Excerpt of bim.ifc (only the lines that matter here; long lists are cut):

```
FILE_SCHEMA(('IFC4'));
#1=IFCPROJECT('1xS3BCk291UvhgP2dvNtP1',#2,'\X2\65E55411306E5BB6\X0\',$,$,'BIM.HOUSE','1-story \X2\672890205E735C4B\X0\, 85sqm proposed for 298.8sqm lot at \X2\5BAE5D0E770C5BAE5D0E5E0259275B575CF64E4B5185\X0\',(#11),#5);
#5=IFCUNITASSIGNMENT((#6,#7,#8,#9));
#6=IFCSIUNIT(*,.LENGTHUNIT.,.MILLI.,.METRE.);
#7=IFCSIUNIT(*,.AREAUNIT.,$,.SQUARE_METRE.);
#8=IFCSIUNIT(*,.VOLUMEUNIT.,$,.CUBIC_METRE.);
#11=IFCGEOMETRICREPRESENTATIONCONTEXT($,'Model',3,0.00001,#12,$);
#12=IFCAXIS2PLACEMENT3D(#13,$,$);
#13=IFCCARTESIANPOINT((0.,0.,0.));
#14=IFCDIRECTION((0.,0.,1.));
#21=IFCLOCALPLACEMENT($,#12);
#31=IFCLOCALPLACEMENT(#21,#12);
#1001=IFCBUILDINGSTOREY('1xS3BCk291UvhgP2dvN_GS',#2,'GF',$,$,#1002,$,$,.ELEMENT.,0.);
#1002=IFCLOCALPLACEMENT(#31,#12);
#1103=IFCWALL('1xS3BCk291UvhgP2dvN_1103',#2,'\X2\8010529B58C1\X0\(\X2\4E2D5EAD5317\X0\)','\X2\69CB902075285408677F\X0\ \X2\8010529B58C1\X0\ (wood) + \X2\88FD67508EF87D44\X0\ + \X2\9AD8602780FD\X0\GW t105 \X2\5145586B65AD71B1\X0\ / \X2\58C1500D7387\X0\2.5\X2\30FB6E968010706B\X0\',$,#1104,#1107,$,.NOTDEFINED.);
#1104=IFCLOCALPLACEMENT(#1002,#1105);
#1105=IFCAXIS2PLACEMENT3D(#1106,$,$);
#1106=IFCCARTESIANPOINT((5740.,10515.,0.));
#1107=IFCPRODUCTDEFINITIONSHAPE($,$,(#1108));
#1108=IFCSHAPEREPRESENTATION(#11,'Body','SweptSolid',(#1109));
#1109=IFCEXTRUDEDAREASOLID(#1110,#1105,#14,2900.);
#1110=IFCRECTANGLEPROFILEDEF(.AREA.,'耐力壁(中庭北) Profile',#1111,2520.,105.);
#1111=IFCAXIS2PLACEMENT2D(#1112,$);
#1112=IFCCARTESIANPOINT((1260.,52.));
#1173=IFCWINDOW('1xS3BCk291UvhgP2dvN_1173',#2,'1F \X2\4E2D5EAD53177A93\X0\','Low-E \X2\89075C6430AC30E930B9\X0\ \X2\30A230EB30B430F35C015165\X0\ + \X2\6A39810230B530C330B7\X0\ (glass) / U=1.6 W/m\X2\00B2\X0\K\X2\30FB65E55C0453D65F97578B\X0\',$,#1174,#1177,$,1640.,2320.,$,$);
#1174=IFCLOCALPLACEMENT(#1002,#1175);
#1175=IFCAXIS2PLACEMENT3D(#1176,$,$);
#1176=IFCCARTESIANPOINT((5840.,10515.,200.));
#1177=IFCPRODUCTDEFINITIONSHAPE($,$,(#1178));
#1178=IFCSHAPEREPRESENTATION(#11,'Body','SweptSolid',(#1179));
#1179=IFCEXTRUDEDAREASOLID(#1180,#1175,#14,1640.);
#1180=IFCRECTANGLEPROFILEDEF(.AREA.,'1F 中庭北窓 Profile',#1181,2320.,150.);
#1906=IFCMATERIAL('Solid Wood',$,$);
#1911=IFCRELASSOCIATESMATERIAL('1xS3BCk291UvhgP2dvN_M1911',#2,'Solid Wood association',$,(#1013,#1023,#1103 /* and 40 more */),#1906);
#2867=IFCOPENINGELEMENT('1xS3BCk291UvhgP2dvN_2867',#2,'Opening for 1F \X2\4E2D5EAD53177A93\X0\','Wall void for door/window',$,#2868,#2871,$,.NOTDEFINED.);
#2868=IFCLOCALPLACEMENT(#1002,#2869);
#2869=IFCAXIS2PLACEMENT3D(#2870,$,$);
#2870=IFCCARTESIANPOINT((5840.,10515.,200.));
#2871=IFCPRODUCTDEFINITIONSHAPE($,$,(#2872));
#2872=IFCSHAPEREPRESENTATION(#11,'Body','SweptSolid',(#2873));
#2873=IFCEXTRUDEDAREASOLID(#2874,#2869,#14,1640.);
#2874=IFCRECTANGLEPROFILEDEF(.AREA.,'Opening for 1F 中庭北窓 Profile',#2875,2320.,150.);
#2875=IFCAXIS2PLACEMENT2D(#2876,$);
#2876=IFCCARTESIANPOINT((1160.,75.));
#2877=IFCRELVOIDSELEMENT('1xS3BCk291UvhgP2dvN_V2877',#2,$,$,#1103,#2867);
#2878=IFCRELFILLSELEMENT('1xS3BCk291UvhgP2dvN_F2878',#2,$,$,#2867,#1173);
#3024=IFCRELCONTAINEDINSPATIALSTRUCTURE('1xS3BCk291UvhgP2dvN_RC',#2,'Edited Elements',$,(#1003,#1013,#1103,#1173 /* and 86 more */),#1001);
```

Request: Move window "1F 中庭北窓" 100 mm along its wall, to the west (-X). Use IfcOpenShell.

```python
import ifcopenshell
import ifcopenshell.api.geometry
import ifcopenshell.util.placement

model = ifcopenshell.open("bim.ifc")

window = model.by_guid("1xS3BCk291UvhgP2dvN_1173")
opening = window.FillsVoids[0].RelatingOpeningElement
wall = opening.VoidsElements[0].RelatingBuildingElement

wall_matrix = ifcopenshell.util.placement.get_local_placement(wall.ObjectPlacement)
shift = wall_matrix[:3, 0] * -100.0
before = ifcopenshell.util.placement.get_local_placement(window.ObjectPlacement)[:3, 3].copy()

# The window is not placed relative to its opening, so move both.
for product in (opening, window):
    matrix = ifcopenshell.util.placement.get_local_placement(product.ObjectPlacement)
    matrix[:3, 3] += shift
    ifcopenshell.api.geometry.edit_object_placement(model, product=product, matrix=matrix, is_si=False)

after = ifcopenshell.util.placement.get_local_placement(window.ObjectPlacement)[:3, 3]
print("window moved by", (after - before).round(3) + 0.0)

model.write("bim_updated.ifc")
```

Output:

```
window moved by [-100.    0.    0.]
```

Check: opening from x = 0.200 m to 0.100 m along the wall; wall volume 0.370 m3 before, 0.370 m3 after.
